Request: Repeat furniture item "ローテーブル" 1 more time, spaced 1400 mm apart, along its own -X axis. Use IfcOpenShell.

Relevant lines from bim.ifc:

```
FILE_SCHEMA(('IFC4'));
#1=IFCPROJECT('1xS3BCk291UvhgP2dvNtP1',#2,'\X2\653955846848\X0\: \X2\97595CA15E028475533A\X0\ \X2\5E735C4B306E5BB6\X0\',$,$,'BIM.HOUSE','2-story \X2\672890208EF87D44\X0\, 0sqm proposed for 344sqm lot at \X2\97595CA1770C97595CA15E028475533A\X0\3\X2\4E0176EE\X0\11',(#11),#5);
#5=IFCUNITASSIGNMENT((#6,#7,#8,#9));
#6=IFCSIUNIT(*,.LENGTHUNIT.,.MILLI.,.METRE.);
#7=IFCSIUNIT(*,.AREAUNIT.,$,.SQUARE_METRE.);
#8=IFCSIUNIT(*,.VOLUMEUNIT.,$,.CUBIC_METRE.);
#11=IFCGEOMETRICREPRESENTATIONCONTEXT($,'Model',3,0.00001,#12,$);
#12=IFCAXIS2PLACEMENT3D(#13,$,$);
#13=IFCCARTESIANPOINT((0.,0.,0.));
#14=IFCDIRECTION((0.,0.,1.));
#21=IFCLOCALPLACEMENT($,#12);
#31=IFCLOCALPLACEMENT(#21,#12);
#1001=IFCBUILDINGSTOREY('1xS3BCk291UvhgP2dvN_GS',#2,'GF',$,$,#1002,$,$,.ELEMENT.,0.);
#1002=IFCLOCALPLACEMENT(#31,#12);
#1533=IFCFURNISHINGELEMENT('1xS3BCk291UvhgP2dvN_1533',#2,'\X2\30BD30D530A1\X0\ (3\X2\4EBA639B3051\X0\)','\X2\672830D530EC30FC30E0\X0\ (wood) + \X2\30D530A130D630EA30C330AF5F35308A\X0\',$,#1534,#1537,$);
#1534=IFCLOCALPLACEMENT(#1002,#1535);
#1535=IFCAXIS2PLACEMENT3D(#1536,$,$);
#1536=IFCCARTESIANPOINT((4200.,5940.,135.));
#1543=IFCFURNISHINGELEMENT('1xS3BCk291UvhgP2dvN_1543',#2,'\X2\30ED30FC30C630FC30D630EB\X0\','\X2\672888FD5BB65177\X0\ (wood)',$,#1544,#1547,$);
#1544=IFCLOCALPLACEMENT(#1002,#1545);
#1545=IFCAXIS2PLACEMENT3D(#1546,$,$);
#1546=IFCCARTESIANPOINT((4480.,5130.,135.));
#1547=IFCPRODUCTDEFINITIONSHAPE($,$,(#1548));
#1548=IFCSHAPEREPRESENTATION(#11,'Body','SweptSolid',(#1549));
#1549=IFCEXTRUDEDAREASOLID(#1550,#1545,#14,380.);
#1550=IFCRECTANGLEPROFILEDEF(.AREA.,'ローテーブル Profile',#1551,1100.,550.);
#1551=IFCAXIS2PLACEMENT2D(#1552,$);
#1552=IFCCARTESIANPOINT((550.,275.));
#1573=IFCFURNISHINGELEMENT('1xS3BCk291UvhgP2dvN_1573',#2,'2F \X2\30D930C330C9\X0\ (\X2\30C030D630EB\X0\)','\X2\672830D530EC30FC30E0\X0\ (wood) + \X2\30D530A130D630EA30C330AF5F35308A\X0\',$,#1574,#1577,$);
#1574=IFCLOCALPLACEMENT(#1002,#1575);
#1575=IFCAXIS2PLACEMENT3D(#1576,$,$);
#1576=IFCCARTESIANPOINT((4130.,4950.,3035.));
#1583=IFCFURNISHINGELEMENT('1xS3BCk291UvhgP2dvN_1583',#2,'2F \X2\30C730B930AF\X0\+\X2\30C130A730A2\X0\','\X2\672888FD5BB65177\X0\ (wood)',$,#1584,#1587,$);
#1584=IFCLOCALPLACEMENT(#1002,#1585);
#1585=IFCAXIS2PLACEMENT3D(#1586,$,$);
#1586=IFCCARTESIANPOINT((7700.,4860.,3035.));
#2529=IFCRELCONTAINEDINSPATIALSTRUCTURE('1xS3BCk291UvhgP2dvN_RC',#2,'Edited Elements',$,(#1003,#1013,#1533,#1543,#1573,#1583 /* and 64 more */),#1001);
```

```python
import ifcopenshell
import ifcopenshell.api.geometry
import ifcopenshell.api.root
import ifcopenshell.util.element
import ifcopenshell.util.placement

model = ifcopenshell.open("bim.ifc")


def reuse_history(source, copy):
    """copy_class also copies each property set's owner history, people and application; keep the originals."""
    for rel in copy.IsDefinedBy:
        if rel.is_a("IfcRelDefinesByProperties") and (history := rel.RelatingPropertyDefinition.OwnerHistory):
            rel.RelatingPropertyDefinition.OwnerHistory = source.OwnerHistory
            ifcopenshell.util.element.remove_deep2(model, history)


source = model.by_id(1543)
base = ifcopenshell.util.placement.get_local_placement(source.ObjectPlacement)
step = -base[:3, 0] * 1400.0

for i in range(1, 2):
    copy = ifcopenshell.api.root.copy_class(model, product=source)
    copy.Representation = ifcopenshell.util.element.copy_deep(
        model, source.Representation, exclude=["IfcGeometricRepresentationContext", "IfcRepresentationMap"]
    )
    reuse_history(source, copy)
    matrix = base.copy()
    matrix[:3, 3] += i * step
    print("added at", matrix[:3, 3].round(3) + 0.0)
    ifcopenshell.api.geometry.edit_object_placement(model, product=copy, matrix=matrix, is_si=False)

model.write("bim_edited.ifc")
```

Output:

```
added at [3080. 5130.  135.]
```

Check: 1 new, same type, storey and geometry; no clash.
